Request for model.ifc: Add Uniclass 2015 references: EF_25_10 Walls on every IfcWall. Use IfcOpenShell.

First a look at what the model holds.

```python
import ifcopenshell

model = ifcopenshell.open("model.ifc")
print(model.schema)
print("classifications:", [c.Name for c in model.by_type("IfcClassification")])
for ifc_class in ("IfcDoor", "IfcRoof", "IfcStair", "IfcWall", "IfcWindow"):
    print(ifc_class, len(model.by_type(ifc_class)))
```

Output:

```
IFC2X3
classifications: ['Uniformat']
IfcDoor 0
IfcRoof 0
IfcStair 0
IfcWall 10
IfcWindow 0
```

```python
import ifcopenshell
import ifcopenshell.api.classification

model = ifcopenshell.open("model.ifc")

# IFC2X3 requires Source and Edition and has no link from the project to the system.
system = model.create_entity("IfcClassification", Source="NBS", Edition="2015", Name="Uniclass 2015")

codes = {
    "IfcWall": ("EF_25_10", "Walls"),
}
for ifc_class, (code, name) in codes.items():
    products = model.by_type(ifc_class)
    ifcopenshell.api.classification.add_reference(
        model, products=products, classification=system, identification=code, name=name
    )
    print(code, len(products))

model.write("model-out.ifc")
```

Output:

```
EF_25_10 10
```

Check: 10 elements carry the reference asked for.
